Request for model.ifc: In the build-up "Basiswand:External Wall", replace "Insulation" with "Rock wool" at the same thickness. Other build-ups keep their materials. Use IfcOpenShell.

First a look at what the model holds.

```python
import ifcopenshell
import ifcopenshell.util.element

model = ifcopenshell.open("model.ifc")
print(model.schema)
for layer_set in model.by_type("IfcMaterialLayerSet"):
    if layer_set.LayerSetName == "Basiswand:External Wall":
        for layer in layer_set.MaterialLayers:
            print(layer.id(), layer.Material and layer.Material.Name, layer.LayerThickness, sep=" | ")
        print(len(ifcopenshell.util.element.get_elements_by_material(model, layer_set)), "elements and types use it")
print(sorted(m.Name for m in model.by_type("IfcMaterial") if m.Name)[:60])
```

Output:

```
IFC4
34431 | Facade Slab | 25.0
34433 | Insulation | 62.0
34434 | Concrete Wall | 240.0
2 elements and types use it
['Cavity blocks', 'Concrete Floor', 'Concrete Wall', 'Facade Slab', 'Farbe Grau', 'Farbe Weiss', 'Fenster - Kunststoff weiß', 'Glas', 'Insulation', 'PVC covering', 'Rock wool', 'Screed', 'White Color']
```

```python
import ifcopenshell
import ifcopenshell.api.material

model = ifcopenshell.open("model.ifc")

layer_set = next(s for s in model.by_type("IfcMaterialLayerSet") if s.LayerSetName == "Basiswand:External Wall")
layer = next(l for l in layer_set.MaterialLayers if l.Material and l.Material.Name == "Insulation")
material = next(m for m in model.by_type("IfcMaterial") if m.Name == "Rock wool")

# Point this one layer at the other material; renaming the old one would change it everywhere.
ifcopenshell.api.material.edit_layer(model, layer=layer, attributes={}, material=material)

print([l.Material.Name if l.Material else None for l in layer_set.MaterialLayers])

model.write("model-out.ifc")
```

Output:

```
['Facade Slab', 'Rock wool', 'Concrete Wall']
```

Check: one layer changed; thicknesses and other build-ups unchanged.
